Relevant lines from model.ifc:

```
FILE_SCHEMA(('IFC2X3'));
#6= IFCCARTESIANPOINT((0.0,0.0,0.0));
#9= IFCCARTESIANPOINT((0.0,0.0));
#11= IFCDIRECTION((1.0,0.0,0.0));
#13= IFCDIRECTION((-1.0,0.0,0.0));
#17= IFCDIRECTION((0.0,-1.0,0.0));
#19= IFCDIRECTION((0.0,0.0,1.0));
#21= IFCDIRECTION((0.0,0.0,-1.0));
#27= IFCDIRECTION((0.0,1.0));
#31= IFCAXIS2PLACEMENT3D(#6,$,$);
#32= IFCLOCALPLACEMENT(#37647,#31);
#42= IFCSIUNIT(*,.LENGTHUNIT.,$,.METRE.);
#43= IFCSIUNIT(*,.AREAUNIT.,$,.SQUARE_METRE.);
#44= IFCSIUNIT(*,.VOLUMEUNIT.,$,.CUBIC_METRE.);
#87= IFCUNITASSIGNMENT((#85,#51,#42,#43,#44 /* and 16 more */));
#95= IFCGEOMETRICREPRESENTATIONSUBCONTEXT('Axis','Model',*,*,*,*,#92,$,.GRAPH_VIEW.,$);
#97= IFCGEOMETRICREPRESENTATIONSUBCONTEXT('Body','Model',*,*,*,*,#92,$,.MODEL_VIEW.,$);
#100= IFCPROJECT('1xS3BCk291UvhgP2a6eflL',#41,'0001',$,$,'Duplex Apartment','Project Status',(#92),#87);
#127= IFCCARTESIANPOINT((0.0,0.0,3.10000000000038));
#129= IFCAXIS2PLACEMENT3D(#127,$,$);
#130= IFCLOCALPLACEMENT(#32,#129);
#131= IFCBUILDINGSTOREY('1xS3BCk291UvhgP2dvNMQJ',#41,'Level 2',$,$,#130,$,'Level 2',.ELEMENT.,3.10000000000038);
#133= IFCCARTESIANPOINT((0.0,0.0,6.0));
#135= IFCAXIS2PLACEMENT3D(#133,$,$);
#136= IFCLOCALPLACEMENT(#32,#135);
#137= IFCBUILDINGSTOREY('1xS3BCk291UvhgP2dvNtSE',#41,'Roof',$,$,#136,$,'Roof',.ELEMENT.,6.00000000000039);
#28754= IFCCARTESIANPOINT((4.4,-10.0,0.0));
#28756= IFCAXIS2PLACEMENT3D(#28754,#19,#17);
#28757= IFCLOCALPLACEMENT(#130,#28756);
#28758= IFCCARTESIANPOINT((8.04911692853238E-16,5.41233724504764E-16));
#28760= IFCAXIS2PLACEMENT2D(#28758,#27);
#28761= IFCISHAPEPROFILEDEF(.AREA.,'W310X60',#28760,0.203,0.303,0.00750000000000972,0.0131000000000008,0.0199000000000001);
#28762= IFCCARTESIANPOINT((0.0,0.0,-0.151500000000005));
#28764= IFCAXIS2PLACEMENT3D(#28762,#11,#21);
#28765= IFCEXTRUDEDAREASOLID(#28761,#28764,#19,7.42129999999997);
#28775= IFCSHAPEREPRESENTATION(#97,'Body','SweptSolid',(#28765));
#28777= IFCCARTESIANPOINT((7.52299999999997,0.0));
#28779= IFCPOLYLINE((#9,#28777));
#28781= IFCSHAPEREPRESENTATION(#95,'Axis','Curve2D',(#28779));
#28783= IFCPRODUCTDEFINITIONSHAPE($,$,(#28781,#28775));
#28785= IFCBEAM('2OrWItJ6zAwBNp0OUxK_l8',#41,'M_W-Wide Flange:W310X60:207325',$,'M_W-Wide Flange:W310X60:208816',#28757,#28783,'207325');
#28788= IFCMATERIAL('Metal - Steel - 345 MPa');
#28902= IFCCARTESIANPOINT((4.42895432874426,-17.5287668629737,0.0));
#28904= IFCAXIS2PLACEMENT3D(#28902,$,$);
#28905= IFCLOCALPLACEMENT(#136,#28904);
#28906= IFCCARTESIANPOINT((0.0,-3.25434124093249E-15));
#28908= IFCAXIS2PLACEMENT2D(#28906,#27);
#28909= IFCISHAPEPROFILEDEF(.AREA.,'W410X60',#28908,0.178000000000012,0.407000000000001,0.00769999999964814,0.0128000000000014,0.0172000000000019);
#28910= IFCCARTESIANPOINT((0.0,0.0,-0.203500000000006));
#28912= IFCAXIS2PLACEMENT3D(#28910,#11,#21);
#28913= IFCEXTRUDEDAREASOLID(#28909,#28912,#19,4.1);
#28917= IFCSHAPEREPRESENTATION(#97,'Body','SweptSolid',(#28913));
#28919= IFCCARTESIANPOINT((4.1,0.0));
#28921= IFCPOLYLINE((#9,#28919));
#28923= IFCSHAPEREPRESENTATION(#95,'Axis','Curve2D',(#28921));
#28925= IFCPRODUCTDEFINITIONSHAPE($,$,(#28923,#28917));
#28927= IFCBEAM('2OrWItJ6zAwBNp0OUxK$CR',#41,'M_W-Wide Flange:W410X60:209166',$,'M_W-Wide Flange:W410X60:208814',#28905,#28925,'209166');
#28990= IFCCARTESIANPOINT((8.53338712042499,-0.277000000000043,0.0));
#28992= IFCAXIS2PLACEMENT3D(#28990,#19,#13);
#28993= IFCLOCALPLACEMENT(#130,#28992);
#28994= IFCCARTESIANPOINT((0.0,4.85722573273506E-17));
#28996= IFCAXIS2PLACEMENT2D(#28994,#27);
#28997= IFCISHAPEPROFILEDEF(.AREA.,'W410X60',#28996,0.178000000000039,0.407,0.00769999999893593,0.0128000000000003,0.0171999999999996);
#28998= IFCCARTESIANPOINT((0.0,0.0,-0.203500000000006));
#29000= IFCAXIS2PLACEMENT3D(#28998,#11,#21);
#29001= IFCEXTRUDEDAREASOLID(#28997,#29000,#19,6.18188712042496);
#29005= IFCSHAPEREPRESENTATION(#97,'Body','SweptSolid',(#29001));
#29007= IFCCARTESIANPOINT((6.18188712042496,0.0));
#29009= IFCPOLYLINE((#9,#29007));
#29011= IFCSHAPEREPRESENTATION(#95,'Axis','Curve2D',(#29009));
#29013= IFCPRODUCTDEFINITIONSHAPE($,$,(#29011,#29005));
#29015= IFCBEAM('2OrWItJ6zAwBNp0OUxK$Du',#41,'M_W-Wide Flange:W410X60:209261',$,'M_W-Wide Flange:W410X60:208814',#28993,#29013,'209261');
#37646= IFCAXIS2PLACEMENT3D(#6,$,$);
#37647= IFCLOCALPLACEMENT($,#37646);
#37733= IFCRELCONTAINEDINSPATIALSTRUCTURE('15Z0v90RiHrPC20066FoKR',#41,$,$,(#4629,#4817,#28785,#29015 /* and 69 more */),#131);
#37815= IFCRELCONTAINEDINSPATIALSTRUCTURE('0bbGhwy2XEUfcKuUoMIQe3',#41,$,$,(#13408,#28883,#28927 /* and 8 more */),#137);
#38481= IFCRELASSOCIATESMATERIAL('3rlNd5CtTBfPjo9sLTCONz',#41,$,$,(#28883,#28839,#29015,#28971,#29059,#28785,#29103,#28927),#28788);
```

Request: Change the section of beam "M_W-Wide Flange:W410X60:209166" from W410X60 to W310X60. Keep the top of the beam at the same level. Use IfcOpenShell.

```python
import ifcopenshell
import ifcopenshell.util.element
import ifcopenshell.util.representation

model = ifcopenshell.open("model.ifc")

member = model.by_guid("2OrWItJ6zAwBNp0OUxK$CR")
source = next(p for p in model.by_type("IfcIShapeProfileDef") if p.ProfileName == "W310X60")

body = ifcopenshell.util.representation.get_representation(member, "Model", "Body")
solid = body.Items[0]
old_profile = solid.SweptArea

# Copy the section's sizes but keep this member's own profile position.
profile = ifcopenshell.util.element.copy(model, source)
# Profiles are centred, so shift by half the change in depth to hold the top.
shift = (old_profile.OverallDepth - profile.OverallDepth) / 2
x, y = old_profile.Position.Location.Coordinates
up = (-1.0, 0.0)  # upwards, in the solid's own plane
location = model.createIfcCartesianPoint((x + up[0] * shift, y + up[1] * shift))
profile.Position = model.createIfcAxis2Placement2D(location, old_profile.Position.RefDirection)
solid.SweptArea = profile
if not model.get_total_inverses(old_profile):
    ifcopenshell.util.element.remove_deep2(model, old_profile)
member.Name = member.Name.replace("W410X60", "W310X60")
member.ObjectType = member.ObjectType.replace("W410X60", "W310X60")

print(solid.SweptArea)

model.write("model_updated.ifc")
```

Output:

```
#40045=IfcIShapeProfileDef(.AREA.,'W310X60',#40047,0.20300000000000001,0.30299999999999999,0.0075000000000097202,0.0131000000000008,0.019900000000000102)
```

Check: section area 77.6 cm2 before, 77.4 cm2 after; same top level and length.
